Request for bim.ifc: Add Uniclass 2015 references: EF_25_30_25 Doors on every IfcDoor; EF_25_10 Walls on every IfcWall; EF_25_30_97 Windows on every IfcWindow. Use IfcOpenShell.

First a look at what the model holds.

```python
import ifcopenshell

model = ifcopenshell.open("bim.ifc")
print(model.schema)
print("classifications:", [c.Name for c in model.by_type("IfcClassification")])
for ifc_class in ("IfcDoor", "IfcRoof", "IfcStair", "IfcWall", "IfcWindow"):
    print(ifc_class, len(model.by_type(ifc_class)))
```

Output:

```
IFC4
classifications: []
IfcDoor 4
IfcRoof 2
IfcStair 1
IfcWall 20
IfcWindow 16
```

```python
import ifcopenshell
import ifcopenshell.api.classification

model = ifcopenshell.open("bim.ifc")

system = ifcopenshell.api.classification.add_classification(model, classification="Uniclass 2015")

codes = {
    "IfcDoor": ("EF_25_30_25", "Doors"),
    "IfcWall": ("EF_25_10", "Walls"),
    "IfcWindow": ("EF_25_30_97", "Windows"),
}
for ifc_class, (code, name) in codes.items():
    products = model.by_type(ifc_class)
    ifcopenshell.api.classification.add_reference(
        model, products=products, classification=system, identification=code, name=name
    )
    print(code, len(products))

model.write("bim_updated.ifc")
```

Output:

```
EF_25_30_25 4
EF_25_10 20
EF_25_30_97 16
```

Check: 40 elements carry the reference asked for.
